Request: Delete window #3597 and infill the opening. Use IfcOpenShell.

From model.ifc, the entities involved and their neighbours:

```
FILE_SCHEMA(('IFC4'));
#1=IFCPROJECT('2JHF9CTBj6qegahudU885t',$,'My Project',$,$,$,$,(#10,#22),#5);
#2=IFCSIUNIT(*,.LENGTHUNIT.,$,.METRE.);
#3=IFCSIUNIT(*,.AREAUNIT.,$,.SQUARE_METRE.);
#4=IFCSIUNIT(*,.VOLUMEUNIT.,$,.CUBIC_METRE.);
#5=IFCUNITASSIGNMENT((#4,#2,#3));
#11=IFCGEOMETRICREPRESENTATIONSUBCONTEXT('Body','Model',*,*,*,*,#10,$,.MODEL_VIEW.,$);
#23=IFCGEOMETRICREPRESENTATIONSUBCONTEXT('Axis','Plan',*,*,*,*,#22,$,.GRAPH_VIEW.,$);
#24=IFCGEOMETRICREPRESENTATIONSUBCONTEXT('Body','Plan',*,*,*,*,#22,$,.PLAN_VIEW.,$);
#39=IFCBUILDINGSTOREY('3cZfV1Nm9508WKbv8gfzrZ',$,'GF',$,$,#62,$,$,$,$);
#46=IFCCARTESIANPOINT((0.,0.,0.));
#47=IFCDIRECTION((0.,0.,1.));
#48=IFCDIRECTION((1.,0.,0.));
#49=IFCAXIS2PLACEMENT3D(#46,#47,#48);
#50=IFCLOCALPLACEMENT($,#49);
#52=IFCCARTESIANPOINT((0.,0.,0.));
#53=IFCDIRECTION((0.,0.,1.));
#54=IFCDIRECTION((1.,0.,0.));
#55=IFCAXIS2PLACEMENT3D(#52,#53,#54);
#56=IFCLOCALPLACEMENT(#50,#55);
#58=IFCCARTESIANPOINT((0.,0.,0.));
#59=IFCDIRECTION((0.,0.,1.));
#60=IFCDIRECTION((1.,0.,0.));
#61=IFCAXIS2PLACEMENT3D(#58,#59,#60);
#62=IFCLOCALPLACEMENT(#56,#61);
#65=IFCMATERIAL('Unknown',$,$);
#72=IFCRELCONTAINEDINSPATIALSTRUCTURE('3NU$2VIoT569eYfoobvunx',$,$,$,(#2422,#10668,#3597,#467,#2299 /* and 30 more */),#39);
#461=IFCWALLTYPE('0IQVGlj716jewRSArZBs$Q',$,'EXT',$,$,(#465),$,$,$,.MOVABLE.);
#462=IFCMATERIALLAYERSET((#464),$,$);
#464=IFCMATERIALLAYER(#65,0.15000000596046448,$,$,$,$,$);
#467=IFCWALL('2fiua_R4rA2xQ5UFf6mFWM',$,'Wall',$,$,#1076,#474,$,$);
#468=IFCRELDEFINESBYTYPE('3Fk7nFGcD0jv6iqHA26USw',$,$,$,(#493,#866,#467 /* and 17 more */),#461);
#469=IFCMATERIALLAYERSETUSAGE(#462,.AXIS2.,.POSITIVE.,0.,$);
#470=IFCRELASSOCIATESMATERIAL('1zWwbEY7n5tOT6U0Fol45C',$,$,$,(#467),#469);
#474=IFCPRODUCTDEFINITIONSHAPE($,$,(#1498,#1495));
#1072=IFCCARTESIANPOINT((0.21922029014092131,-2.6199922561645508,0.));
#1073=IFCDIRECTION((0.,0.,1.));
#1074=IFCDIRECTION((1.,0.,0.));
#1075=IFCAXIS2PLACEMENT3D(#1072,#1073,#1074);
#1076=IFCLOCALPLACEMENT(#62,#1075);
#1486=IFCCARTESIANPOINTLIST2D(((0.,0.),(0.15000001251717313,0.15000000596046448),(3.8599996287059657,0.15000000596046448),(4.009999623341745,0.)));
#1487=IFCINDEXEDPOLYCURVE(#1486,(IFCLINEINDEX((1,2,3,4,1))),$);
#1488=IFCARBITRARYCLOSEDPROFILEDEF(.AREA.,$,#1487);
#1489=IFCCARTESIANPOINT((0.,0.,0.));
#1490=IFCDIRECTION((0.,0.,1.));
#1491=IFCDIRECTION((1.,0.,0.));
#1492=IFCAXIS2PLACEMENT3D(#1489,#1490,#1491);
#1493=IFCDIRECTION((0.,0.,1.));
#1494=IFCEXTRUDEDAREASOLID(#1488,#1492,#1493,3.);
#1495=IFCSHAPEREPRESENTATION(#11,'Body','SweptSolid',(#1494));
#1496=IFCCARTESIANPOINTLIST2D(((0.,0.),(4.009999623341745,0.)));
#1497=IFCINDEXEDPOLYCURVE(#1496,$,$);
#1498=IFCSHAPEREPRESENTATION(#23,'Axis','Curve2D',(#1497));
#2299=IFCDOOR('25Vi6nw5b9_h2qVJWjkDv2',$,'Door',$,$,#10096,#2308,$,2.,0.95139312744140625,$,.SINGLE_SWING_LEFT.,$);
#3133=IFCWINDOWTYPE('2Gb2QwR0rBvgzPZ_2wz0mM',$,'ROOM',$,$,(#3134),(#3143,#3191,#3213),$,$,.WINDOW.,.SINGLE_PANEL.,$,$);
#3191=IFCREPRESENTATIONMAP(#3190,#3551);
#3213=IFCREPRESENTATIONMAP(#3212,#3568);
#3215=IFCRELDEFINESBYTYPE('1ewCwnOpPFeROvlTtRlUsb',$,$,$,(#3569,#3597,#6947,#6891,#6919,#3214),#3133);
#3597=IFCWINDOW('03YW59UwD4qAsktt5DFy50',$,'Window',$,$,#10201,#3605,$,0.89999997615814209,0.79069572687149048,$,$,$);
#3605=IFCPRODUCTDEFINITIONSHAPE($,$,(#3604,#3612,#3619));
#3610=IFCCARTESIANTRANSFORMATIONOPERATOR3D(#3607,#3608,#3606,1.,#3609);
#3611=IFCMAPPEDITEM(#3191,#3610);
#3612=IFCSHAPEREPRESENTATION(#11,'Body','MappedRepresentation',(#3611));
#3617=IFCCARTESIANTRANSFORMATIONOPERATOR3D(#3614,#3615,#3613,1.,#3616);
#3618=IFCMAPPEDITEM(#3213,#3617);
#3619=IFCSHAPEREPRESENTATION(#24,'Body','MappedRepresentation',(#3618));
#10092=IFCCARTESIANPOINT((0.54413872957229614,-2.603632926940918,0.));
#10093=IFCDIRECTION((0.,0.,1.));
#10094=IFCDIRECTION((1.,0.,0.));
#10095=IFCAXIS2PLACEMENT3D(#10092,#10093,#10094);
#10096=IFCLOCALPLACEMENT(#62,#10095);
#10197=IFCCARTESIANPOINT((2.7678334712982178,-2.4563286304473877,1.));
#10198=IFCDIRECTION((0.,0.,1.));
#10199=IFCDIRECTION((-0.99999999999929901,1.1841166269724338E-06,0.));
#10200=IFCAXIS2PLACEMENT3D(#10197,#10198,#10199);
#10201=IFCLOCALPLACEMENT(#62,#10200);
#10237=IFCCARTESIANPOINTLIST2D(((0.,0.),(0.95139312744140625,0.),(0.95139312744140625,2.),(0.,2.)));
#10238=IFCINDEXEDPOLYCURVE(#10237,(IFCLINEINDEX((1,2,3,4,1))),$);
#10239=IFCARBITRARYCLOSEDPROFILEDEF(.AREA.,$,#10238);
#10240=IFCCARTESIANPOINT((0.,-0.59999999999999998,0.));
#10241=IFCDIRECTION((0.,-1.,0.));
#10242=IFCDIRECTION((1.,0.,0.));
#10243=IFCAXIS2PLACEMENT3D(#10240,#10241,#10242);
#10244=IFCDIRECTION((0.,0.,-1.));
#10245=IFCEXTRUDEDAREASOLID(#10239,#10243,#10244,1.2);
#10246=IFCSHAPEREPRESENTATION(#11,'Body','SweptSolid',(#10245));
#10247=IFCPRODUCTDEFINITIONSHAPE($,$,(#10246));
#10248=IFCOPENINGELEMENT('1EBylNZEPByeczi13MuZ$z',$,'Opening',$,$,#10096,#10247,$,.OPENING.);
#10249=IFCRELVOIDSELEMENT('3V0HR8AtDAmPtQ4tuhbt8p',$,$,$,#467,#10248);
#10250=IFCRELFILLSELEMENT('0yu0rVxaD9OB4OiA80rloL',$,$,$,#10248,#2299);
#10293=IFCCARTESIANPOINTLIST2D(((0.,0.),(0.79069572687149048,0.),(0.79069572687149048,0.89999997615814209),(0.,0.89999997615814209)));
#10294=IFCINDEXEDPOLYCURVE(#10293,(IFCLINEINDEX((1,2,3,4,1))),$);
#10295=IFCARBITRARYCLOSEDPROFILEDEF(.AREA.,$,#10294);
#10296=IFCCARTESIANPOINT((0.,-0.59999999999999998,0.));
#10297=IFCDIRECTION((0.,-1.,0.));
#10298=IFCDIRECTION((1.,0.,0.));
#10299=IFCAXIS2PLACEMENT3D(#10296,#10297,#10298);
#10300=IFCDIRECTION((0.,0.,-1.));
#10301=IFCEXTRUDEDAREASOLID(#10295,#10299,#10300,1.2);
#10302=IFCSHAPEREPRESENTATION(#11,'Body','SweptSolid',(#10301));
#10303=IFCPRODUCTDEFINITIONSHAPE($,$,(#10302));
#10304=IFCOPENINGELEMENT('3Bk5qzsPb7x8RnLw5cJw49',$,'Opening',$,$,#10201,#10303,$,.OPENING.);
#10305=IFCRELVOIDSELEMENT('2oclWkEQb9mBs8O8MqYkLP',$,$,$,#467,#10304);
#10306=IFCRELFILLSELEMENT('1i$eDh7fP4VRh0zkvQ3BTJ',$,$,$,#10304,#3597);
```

```python
import ifcopenshell
import ifcopenshell.api.feature
import ifcopenshell.api.root
import ifcopenshell.geom
import ifcopenshell.util.shape

model = ifcopenshell.open("model.ifc")
settings = ifcopenshell.geom.settings()


def volume(element):
    """Net volume in cubic metres, openings subtracted."""
    shape = ifcopenshell.geom.create_shape(settings, element)
    return ifcopenshell.util.shape.get_volume(shape.geometry)


window = model.by_guid("03YW59UwD4qAsktt5DFy50")
opening = window.FillsVoids[0].RelatingOpeningElement
wall = opening.VoidsElements[0].RelatingBuildingElement
before = volume(wall)

ifcopenshell.api.root.remove_product(model, product=window)
ifcopenshell.api.feature.remove_feature(model, feature=opening)

after = volume(wall)

print(f"wall volume {before:.3f} -> {after:.3f} m3")

model.write("model-out.ifc")
```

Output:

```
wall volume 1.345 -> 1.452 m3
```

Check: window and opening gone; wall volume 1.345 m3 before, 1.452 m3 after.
